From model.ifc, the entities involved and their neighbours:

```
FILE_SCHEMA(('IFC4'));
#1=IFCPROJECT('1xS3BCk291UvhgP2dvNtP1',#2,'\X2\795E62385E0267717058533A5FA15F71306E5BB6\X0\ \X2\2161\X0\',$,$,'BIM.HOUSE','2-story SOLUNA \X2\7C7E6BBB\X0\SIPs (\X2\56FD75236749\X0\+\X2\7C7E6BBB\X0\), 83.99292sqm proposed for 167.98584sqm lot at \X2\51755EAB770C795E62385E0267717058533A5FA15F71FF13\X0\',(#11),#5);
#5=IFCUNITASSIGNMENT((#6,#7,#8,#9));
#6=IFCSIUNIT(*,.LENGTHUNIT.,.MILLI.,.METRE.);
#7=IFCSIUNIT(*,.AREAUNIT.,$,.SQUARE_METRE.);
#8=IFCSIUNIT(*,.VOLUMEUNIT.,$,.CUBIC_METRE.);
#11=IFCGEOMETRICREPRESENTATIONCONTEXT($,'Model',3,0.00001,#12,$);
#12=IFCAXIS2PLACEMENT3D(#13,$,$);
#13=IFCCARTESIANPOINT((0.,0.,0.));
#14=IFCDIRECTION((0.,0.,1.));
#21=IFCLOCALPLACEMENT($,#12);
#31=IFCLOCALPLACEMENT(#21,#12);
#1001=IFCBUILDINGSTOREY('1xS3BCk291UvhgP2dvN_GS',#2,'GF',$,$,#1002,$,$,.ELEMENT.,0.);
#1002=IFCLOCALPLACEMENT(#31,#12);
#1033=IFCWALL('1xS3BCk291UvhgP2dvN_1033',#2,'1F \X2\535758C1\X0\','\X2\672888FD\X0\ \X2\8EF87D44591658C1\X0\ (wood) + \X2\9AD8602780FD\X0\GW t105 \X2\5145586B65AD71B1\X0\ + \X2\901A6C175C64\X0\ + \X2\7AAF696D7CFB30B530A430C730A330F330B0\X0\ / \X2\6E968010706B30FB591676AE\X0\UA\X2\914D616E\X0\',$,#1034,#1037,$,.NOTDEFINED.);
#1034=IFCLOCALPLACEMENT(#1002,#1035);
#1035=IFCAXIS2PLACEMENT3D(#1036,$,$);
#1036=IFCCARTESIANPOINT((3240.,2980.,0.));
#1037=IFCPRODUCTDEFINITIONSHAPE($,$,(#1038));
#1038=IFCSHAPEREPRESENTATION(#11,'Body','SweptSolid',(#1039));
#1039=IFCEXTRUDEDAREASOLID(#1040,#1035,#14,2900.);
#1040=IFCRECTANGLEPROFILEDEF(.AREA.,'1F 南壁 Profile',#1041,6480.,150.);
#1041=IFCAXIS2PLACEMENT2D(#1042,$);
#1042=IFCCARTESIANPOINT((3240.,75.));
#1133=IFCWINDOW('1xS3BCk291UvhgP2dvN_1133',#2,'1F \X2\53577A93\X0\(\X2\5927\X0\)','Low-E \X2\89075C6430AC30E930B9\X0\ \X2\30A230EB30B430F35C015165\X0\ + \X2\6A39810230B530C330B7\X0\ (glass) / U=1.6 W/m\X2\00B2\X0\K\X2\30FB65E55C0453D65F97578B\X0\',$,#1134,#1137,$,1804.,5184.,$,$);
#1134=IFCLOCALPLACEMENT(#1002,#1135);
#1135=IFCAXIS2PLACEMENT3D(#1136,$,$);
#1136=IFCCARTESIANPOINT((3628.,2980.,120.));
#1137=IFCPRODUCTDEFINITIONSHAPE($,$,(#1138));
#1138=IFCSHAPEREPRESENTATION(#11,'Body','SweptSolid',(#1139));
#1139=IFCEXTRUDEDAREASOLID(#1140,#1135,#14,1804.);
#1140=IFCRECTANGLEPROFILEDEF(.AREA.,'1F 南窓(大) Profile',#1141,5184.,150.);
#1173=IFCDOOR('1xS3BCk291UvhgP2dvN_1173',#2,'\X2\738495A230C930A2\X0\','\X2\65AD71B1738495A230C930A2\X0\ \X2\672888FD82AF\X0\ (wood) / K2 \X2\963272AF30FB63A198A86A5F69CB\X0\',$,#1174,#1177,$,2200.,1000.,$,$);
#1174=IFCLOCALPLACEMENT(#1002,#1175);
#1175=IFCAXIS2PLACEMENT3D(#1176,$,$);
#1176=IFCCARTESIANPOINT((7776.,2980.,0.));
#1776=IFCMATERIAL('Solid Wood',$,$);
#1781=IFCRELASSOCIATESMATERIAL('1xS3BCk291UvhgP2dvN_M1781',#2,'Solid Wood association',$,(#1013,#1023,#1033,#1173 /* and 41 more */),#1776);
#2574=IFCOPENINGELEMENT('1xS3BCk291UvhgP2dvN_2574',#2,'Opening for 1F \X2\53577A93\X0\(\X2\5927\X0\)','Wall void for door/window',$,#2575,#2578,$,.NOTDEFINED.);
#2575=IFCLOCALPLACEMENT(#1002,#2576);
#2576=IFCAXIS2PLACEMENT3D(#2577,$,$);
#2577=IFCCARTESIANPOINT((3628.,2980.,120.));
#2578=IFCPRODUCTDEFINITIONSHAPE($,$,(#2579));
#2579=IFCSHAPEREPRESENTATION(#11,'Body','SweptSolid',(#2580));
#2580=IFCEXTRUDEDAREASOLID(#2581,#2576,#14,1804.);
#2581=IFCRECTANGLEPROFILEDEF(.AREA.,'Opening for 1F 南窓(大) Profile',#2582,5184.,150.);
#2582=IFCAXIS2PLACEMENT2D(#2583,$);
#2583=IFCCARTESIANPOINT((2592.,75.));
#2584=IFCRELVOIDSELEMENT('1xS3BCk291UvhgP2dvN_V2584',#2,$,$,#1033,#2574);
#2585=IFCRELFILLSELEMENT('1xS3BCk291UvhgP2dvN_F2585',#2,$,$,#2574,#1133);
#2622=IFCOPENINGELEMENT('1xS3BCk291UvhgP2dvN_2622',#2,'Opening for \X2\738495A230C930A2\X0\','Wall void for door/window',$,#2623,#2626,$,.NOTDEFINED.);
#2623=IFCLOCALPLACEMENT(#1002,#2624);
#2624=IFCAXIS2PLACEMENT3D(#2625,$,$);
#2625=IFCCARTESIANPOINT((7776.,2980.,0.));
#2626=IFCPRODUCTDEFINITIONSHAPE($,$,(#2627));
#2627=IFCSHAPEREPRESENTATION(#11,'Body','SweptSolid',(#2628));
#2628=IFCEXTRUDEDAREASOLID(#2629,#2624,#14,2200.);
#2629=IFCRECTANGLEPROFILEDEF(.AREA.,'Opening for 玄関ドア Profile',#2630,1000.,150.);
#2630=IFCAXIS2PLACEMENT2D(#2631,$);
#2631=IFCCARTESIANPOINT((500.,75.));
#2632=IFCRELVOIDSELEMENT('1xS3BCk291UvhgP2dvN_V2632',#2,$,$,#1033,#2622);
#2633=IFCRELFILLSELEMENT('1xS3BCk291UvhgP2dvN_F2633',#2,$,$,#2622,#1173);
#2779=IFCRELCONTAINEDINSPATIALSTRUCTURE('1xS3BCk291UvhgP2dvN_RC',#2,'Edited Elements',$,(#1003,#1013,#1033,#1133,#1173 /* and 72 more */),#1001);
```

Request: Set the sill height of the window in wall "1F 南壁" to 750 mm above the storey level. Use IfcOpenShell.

```python
import numpy as np
import ifcopenshell
import ifcopenshell.api.geometry
import ifcopenshell.geom
import ifcopenshell.util.element
import ifcopenshell.util.placement
import ifcopenshell.util.shape
import ifcopenshell.util.unit

model = ifcopenshell.open("model.ifc")
unit_scale = ifcopenshell.util.unit.calculate_unit_scale(model)

window = model.by_guid("1xS3BCk291UvhgP2dvN_1133")
opening = window.FillsVoids[0].RelatingOpeningElement
storey = ifcopenshell.util.element.get_container(window, ifc_class="IfcBuildingStorey")
level = ifcopenshell.util.placement.get_local_placement(storey.ObjectPlacement)[2, 3]

# The opening's origin need not be at the sill, so measure its lowest point.
shape = ifcopenshell.geom.create_shape(ifcopenshell.geom.settings(), opening)
bottom = ifcopenshell.util.shape.get_shape_bottom_elevation(shape, shape.geometry) / unit_scale
dz = level + 750.0 - bottom

shift = np.array([0.0, 0.0, dz])
# The window is not placed relative to its opening, so move both.
for product in (opening, window):
    matrix = ifcopenshell.util.placement.get_local_placement(product.ObjectPlacement)
    matrix[:3, 3] += shift
    ifcopenshell.api.geometry.edit_object_placement(model, product=product, matrix=matrix, is_si=False)

print(f"moved by {dz * unit_scale:+.3f} m")

model.write("model_edited.ifc")
```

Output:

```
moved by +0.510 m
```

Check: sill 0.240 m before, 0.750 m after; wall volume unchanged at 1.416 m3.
